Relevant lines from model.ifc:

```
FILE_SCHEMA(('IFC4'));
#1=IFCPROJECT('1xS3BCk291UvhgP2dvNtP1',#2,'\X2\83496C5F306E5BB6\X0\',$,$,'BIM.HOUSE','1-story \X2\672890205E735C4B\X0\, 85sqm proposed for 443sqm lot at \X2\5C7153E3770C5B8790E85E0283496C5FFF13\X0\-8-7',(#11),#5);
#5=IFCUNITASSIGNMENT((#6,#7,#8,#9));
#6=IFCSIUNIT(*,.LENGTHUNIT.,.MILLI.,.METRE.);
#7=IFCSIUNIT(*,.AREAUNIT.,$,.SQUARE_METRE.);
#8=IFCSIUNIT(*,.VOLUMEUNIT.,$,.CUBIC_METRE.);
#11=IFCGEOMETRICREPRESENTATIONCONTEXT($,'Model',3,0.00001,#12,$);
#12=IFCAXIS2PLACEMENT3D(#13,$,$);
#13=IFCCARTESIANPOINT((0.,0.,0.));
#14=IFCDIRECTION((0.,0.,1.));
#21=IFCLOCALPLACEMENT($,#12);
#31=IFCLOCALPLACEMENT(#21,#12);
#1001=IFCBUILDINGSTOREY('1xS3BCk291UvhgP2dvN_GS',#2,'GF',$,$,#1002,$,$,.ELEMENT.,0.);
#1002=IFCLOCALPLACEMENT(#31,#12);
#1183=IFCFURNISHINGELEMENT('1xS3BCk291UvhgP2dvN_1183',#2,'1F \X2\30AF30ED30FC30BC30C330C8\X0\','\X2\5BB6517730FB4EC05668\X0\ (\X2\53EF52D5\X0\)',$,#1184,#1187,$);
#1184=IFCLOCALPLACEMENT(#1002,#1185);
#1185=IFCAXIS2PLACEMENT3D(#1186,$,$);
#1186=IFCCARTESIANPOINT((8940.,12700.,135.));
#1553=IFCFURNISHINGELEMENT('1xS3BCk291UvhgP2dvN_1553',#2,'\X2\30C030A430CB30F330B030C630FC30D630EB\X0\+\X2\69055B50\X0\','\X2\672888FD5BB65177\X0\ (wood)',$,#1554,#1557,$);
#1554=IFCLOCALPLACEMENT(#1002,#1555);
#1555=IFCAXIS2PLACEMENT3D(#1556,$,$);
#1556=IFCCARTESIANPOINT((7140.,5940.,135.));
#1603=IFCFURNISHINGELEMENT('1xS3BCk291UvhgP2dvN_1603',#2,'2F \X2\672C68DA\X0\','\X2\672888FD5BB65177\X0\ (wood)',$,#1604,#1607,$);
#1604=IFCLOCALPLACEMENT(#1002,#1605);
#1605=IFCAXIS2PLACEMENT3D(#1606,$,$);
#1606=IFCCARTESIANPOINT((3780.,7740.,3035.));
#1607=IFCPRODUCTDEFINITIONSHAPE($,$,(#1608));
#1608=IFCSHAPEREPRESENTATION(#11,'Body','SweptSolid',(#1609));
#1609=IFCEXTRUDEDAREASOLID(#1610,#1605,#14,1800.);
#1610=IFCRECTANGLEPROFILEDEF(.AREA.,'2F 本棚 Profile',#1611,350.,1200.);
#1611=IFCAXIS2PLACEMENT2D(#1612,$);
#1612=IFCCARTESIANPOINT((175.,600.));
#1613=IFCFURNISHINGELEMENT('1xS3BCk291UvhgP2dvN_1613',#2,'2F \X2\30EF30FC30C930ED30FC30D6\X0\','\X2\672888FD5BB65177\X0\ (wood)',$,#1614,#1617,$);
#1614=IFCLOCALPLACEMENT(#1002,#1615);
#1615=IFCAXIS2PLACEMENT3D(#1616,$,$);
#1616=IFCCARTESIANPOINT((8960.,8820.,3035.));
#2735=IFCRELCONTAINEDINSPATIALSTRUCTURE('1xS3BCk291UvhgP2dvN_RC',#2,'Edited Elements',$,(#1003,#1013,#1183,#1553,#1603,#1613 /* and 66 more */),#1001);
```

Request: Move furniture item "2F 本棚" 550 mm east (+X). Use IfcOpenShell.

```python
import ifcopenshell
import ifcopenshell.api.geometry
import ifcopenshell.util.placement
import ifcopenshell.util.unit

model = ifcopenshell.open("model.ifc")
unit_scale = ifcopenshell.util.unit.calculate_unit_scale(model)

item = model.by_guid("1xS3BCk291UvhgP2dvN_1603")
matrix = ifcopenshell.util.placement.get_local_placement(item.ObjectPlacement)
matrix[0, 3] += 0.55 / unit_scale
ifcopenshell.api.geometry.edit_object_placement(model, product=item, matrix=matrix, is_si=False)

print(ifcopenshell.util.placement.get_local_placement(item.ObjectPlacement).round(3) + 0.0)

model.write("model_updated.ifc")
```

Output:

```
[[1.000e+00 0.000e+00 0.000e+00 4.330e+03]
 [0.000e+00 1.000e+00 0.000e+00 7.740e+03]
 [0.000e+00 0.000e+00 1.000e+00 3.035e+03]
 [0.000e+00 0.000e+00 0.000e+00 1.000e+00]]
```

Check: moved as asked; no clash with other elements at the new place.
